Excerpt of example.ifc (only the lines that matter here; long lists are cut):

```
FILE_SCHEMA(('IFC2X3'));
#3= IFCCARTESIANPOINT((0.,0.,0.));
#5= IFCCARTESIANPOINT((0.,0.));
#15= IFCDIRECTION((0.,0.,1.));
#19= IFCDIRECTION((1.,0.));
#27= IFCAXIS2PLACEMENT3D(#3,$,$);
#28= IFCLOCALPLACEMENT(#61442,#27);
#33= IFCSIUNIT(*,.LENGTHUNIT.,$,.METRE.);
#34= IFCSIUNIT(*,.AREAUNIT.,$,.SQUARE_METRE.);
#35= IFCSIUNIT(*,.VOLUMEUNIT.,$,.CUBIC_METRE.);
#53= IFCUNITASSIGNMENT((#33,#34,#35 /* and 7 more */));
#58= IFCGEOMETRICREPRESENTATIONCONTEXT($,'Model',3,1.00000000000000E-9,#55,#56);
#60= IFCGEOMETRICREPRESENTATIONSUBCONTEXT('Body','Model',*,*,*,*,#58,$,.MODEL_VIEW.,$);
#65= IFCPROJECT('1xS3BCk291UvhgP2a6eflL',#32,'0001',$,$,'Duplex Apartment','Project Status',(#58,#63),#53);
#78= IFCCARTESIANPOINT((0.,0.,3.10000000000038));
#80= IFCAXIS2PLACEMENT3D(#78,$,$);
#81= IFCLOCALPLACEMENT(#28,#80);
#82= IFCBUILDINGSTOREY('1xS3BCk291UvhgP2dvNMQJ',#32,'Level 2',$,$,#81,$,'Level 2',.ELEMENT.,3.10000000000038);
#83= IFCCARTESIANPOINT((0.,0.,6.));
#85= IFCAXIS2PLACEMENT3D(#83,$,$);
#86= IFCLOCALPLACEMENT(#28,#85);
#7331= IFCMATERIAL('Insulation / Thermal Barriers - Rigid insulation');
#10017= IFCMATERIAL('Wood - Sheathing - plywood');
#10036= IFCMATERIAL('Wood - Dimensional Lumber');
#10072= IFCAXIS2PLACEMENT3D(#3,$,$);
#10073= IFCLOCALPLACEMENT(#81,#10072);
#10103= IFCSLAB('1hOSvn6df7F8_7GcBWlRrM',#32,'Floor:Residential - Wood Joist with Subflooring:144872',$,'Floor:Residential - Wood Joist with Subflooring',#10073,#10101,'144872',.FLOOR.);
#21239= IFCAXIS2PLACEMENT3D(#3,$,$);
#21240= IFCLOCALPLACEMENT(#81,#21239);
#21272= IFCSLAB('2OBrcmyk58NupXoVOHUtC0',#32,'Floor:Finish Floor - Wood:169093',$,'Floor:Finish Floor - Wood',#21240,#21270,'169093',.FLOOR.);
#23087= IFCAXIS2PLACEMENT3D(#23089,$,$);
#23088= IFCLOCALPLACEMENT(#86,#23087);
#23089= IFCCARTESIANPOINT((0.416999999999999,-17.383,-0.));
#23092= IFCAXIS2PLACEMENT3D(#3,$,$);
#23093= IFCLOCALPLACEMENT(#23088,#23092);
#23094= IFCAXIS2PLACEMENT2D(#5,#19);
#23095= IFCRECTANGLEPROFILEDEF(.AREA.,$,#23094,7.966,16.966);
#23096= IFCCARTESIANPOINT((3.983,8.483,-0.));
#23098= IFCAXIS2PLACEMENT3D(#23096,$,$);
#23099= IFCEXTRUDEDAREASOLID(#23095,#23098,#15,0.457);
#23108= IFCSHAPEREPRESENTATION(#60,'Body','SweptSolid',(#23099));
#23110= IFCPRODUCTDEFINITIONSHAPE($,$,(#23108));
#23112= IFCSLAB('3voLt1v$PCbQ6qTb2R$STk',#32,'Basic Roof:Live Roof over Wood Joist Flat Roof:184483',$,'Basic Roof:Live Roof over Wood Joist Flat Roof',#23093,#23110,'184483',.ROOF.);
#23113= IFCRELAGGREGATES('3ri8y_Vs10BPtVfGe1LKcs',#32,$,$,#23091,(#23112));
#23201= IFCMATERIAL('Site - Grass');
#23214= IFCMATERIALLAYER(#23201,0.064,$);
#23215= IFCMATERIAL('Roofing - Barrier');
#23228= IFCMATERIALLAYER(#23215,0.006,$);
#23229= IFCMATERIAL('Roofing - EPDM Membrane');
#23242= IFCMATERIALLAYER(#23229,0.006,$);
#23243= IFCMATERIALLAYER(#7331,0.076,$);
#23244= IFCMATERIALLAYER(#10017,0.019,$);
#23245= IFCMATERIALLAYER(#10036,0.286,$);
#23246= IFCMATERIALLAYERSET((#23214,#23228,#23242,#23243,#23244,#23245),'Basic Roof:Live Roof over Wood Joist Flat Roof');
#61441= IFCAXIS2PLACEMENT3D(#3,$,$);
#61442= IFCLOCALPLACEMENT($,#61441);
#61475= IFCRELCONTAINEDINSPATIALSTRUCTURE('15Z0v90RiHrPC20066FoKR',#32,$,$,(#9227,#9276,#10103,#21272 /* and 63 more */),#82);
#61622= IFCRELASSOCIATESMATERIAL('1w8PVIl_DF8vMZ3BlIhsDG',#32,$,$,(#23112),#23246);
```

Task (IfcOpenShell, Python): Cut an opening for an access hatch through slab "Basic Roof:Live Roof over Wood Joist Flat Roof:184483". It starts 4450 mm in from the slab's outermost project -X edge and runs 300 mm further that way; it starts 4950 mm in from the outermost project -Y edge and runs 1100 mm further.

```python
import numpy as np
import ifcopenshell
import ifcopenshell.api.feature
import ifcopenshell.api.geometry
import ifcopenshell.api.root
import ifcopenshell.geom
import ifcopenshell.util.placement
import ifcopenshell.util.representation
import ifcopenshell.util.shape
import ifcopenshell.util.unit

model = ifcopenshell.open("example.ifc")
unit_scale = ifcopenshell.util.unit.calculate_unit_scale(model)
settings = ifcopenshell.geom.settings()


def volume(element):
    """Net volume in cubic metres, openings subtracted."""
    shape = ifcopenshell.geom.create_shape(settings, element)
    return ifcopenshell.util.shape.get_volume(shape.geometry)


slab = model.by_guid("3voLt1v$PCbQ6qTb2R$STk")
before = volume(slab)

# Extent in the slab's own axes, in metres. The edges named are its -X and -Y sides.
slab_shape = ifcopenshell.geom.create_shape(settings, slab)
vertices = ifcopenshell.util.shape.get_vertices(slab_shape.geometry)
x_min, y_min, bottom = vertices.min(axis=0)
top = vertices[:, 2].max()

opening = ifcopenshell.api.root.create_entity(model, ifc_class="IfcOpeningElement", name="Access hatch opening")
context = ifcopenshell.util.representation.get_context(model, "Model", "Body", "MODEL_VIEW")
width, depth = 0.3, 1.1
outline = [(0.0, 0.0), (width, 0.0), (width, depth), (0.0, depth), (0.0, 0.0)]
# Overshoot both faces by 50 mm so the cut is clean.
shape = ifcopenshell.api.geometry.add_slab_representation(
    model, context=context, depth=top - bottom + 0.1, polyline=outline
)
ifcopenshell.api.geometry.assign_representation(model, product=opening, representation=shape)

matrix = ifcopenshell.util.placement.get_local_placement(slab.ObjectPlacement)
matrix[:, 3] = matrix @ np.append(np.array([x_min + 4.45, y_min + 4.95, bottom - 0.05]) / unit_scale, 1.0)
ifcopenshell.api.geometry.edit_object_placement(model, product=opening, matrix=matrix, is_si=False)
ifcopenshell.api.feature.add_feature(model, feature=opening, element=slab)

after = volume(slab)

print(f"slab volume {before:.3f} -> {after:.3f} m3")

model.write("example_updated.ifc")
```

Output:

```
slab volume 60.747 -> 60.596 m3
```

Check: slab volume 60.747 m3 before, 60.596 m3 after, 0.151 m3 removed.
